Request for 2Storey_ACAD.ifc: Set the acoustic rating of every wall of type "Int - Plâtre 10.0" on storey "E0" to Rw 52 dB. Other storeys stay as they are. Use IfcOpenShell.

First a look at what the model holds.

```python
import ifcopenshell
import ifcopenshell.util.element

model = ifcopenshell.open("2Storey_ACAD.ifc")
print(model.schema)
storey = next(s for s in model.by_type("IfcBuildingStorey") if s.Name == "E0")
walls = [e for e in ifcopenshell.util.element.get_decomposition(storey) if e.is_a("IfcWall")]
seen = {}
for e in walls:
    element_type = ifcopenshell.util.element.get_type(e)
    key = (element_type.Name if element_type != e and element_type else None, ifcopenshell.util.element.get_pset(e, "Pset_WallCommon", "AcousticRating"))
    seen[key] = seen.get(key, 0) + 1
for (name, value), count in sorted(seen.items(), key=str):
    print(count, "x", name, "|", value)
```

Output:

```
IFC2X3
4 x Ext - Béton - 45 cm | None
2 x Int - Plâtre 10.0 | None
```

```python
import ifcopenshell
import ifcopenshell.api.pset
import ifcopenshell.util.element

model = ifcopenshell.open("2Storey_ACAD.ifc")

storey = next(s for s in model.by_type("IfcBuildingStorey") if s.Name == "E0")
walls = [e for e in ifcopenshell.util.element.get_decomposition(storey) if e.is_a("IfcWall")]

count = 0
for e in walls:
    element_type = ifcopenshell.util.element.get_type(e)
    if element_type in (None, e) or element_type.Name != "Int - Plâtre 10.0":
        continue
    # add_pset returns the element's existing set when there is one.
    pset = ifcopenshell.api.pset.add_pset(model, product=e, name="Pset_WallCommon")
    ifcopenshell.api.pset.edit_pset(model, pset=pset, properties={"AcousticRating": "Rw 52 dB"})
    count += 1

print(count, "walls updated")

model.write("2Storey_ACAD_edited.ifc")
```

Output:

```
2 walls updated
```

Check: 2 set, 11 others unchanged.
